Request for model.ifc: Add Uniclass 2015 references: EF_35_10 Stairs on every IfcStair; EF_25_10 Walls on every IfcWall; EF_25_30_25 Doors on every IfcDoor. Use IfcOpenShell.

First a look at what the model holds.

```python
import ifcopenshell

model = ifcopenshell.open("model.ifc")
print(model.schema)
print("classifications:", [c.Name for c in model.by_type("IfcClassification")])
for ifc_class in ("IfcDoor", "IfcRoof", "IfcStair", "IfcWall", "IfcWindow"):
    print(ifc_class, len(model.by_type(ifc_class)))
```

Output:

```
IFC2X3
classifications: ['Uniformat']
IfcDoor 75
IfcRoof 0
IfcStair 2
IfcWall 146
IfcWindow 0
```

```python
import ifcopenshell
import ifcopenshell.api.classification

model = ifcopenshell.open("model.ifc")

# IFC2X3 requires Source and Edition and has no link from the project to the system.
system = model.create_entity("IfcClassification", Source="NBS", Edition="2015", Name="Uniclass 2015")

codes = {
    "IfcStair": ("EF_35_10", "Stairs"),
    "IfcWall": ("EF_25_10", "Walls"),
    "IfcDoor": ("EF_25_30_25", "Doors"),
}
for ifc_class, (code, name) in codes.items():
    products = model.by_type(ifc_class)
    ifcopenshell.api.classification.add_reference(
        model, products=products, classification=system, identification=code, name=name
    )
    print(code, len(products))

model.write("model_edited.ifc")
```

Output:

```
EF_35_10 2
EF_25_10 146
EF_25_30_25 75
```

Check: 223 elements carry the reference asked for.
